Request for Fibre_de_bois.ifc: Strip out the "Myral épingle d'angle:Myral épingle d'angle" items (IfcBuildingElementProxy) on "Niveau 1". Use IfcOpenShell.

First a look at what the model holds.

```python
import ifcopenshell
import ifcopenshell.util.element

model = ifcopenshell.open("Fibre_de_bois.ifc")
print(model.schema)
storey = next(s for s in model.by_type("IfcBuildingStorey") if s.Name == "Niveau 1")
proxies = [e for e in ifcopenshell.util.element.get_decomposition(storey) if e.is_a("IfcBuildingElementProxy")]
seen = {}
for e in proxies:
    element_type = ifcopenshell.util.element.get_type(e)
    name = element_type.Name if element_type not in (None, e) else None
    seen[name] = seen.get(name, 0) + 1
for name, count in sorted(seen.items(), key=str):
    print(count, "x", name)
```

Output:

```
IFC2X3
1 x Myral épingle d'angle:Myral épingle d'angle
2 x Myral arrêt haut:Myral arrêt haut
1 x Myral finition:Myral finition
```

```python
import ifcopenshell
import ifcopenshell.api.root
import ifcopenshell.util.element

model = ifcopenshell.open("Fibre_de_bois.ifc")

storey = next(s for s in model.by_type("IfcBuildingStorey") if s.Name == "Niveau 1")
proxies = [e for e in ifcopenshell.util.element.get_decomposition(storey) if e.is_a("IfcBuildingElementProxy")]
targets = [e for e in proxies if (t := ifcopenshell.util.element.get_type(e)) not in (None, e) and t.Name == "Myral épingle d'angle:Myral épingle d'angle"]

for e in targets:
    ifcopenshell.api.root.remove_product(model, product=e)
print(len(targets), "removed")

model.write("Fibre_de_bois_v2.ifc")
```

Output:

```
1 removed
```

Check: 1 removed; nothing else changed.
